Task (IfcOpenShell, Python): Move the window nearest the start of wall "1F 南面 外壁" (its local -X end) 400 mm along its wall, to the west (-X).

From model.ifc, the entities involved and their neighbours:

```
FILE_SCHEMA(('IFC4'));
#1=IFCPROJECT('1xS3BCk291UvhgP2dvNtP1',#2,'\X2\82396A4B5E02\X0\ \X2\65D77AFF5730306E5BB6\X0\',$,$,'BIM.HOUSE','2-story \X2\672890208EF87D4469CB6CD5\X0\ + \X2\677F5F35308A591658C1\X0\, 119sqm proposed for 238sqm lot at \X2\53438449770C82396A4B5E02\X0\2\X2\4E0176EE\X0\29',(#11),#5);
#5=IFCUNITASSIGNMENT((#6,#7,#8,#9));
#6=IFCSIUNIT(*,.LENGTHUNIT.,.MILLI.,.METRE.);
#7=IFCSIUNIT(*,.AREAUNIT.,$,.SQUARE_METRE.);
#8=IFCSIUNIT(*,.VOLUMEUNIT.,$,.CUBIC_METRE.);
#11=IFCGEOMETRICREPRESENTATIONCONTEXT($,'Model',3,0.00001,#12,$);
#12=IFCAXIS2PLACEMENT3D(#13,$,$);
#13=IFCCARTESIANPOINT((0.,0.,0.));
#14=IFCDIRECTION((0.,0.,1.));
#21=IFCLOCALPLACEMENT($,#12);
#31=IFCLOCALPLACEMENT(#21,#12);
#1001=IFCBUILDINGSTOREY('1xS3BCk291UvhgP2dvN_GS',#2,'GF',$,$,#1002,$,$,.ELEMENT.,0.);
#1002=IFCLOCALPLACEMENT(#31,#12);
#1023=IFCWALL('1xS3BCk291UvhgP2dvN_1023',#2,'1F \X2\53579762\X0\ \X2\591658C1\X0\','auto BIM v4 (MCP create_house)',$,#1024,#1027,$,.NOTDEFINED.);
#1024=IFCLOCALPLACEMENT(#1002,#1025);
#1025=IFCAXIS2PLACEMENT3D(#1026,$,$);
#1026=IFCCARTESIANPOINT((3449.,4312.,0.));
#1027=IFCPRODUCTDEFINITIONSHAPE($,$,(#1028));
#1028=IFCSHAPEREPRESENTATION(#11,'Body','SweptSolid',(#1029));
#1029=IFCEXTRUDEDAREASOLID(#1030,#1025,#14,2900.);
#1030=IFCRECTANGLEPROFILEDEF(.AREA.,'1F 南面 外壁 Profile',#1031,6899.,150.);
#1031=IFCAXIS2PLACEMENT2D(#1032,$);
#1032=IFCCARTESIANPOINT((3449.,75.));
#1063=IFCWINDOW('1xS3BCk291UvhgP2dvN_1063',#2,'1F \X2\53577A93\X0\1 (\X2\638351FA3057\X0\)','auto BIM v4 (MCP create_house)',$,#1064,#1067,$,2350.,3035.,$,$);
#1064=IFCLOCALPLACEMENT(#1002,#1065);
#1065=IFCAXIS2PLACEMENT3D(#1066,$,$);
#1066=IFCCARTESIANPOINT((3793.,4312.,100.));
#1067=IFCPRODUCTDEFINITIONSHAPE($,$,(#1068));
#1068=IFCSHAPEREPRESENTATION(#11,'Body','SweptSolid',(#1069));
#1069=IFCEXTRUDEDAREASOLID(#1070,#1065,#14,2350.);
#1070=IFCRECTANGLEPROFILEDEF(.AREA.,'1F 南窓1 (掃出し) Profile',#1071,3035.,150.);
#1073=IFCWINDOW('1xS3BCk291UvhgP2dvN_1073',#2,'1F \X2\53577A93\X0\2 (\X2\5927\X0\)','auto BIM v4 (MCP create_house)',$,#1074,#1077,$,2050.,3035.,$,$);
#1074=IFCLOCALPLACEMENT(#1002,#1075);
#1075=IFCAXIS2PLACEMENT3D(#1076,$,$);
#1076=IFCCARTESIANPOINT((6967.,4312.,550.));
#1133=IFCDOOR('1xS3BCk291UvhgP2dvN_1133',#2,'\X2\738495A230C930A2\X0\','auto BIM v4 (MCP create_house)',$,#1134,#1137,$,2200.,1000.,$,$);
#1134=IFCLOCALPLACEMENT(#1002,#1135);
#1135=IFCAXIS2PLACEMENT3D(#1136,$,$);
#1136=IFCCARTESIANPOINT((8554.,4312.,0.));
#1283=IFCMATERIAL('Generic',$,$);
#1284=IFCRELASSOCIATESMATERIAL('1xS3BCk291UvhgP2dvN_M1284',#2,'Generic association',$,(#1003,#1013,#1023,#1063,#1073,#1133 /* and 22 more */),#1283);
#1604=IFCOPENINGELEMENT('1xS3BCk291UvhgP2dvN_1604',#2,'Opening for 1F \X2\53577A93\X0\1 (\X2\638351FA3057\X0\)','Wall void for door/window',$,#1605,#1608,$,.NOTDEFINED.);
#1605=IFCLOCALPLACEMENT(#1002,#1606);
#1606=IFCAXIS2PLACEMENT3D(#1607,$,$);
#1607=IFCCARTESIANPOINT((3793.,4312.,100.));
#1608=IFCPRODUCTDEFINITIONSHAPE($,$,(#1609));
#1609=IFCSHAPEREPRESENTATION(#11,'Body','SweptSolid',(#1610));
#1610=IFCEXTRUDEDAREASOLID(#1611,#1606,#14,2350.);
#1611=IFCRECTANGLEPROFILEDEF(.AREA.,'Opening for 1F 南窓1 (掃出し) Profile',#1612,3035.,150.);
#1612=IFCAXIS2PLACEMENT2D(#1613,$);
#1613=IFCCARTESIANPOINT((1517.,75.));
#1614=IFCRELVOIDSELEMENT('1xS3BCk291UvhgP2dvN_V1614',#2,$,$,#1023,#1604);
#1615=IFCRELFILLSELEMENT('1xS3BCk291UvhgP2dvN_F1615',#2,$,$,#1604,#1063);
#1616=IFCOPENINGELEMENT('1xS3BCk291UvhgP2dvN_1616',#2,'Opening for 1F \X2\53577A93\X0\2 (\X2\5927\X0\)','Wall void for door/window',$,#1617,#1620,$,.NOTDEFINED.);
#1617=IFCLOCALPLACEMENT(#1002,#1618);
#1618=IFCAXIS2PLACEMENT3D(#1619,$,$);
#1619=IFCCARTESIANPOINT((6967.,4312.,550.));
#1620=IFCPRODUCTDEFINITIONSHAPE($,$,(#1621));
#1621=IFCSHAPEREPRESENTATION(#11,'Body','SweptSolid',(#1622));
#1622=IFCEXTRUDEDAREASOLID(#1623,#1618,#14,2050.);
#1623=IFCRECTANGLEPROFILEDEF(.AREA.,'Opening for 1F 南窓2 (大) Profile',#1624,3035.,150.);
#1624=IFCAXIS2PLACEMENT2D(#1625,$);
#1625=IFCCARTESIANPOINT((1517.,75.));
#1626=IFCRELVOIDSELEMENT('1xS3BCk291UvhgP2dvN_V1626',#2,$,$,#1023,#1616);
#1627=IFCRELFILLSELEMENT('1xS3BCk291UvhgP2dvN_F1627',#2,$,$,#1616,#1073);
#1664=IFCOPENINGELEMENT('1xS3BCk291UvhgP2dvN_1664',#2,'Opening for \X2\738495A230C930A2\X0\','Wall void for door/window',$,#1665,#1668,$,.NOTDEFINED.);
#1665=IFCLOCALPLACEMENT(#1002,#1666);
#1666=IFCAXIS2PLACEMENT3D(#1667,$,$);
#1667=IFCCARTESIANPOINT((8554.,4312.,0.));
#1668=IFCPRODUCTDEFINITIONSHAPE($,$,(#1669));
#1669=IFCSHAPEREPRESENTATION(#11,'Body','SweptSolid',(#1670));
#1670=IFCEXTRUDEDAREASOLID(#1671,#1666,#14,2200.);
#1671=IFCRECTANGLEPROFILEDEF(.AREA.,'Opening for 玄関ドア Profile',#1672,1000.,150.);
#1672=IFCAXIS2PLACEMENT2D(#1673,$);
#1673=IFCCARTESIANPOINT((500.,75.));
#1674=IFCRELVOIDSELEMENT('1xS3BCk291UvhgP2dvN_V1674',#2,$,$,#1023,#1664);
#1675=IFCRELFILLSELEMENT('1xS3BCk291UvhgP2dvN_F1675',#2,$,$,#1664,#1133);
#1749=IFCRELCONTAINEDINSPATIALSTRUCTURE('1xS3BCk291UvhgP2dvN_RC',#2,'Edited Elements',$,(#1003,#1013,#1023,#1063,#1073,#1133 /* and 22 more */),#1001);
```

```python
import ifcopenshell
import ifcopenshell.api.geometry
import ifcopenshell.util.placement

model = ifcopenshell.open("model.ifc")

window = model.by_id(1063)
opening = window.FillsVoids[0].RelatingOpeningElement
wall = opening.VoidsElements[0].RelatingBuildingElement

wall_matrix = ifcopenshell.util.placement.get_local_placement(wall.ObjectPlacement)
shift = wall_matrix[:3, 0] * -400.0
before = ifcopenshell.util.placement.get_local_placement(window.ObjectPlacement)[:3, 3].copy()

# The window is not placed relative to its opening, so move both.
for product in (opening, window):
    matrix = ifcopenshell.util.placement.get_local_placement(product.ObjectPlacement)
    matrix[:3, 3] += shift
    ifcopenshell.api.geometry.edit_object_placement(model, product=product, matrix=matrix, is_si=False)

after = ifcopenshell.util.placement.get_local_placement(window.ObjectPlacement)[:3, 3]
print("window moved by", (after - before).round(3) + 0.0)

model.write("model_edited.ifc")
```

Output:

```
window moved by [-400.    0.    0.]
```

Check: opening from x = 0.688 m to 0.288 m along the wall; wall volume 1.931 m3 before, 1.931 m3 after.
